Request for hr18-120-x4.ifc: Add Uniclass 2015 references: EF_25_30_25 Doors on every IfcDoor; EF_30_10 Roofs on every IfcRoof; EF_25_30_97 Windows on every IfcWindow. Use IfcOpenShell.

First a look at what the model holds.

```python
import ifcopenshell

model = ifcopenshell.open("hr18-120-x4.ifc")
print(model.schema)
print("classifications:", [c.Name for c in model.by_type("IfcClassification")])
for ifc_class in ("IfcDoor", "IfcRoof", "IfcStair", "IfcWall", "IfcWindow"):
    print(ifc_class, len(model.by_type(ifc_class)))
```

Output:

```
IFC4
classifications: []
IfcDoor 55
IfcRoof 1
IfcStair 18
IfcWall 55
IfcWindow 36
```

```python
import ifcopenshell
import ifcopenshell.api.classification

model = ifcopenshell.open("hr18-120-x4.ifc")

system = ifcopenshell.api.classification.add_classification(model, classification="Uniclass 2015")

codes = {
    "IfcDoor": ("EF_25_30_25", "Doors"),
    "IfcRoof": ("EF_30_10", "Roofs"),
    "IfcWindow": ("EF_25_30_97", "Windows"),
}
for ifc_class, (code, name) in codes.items():
    products = model.by_type(ifc_class)
    ifcopenshell.api.classification.add_reference(
        model, products=products, classification=system, identification=code, name=name
    )
    print(code, len(products))

model.write("hr18-120-x4-out.ifc")
```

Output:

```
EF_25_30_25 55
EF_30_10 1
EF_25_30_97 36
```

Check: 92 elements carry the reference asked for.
